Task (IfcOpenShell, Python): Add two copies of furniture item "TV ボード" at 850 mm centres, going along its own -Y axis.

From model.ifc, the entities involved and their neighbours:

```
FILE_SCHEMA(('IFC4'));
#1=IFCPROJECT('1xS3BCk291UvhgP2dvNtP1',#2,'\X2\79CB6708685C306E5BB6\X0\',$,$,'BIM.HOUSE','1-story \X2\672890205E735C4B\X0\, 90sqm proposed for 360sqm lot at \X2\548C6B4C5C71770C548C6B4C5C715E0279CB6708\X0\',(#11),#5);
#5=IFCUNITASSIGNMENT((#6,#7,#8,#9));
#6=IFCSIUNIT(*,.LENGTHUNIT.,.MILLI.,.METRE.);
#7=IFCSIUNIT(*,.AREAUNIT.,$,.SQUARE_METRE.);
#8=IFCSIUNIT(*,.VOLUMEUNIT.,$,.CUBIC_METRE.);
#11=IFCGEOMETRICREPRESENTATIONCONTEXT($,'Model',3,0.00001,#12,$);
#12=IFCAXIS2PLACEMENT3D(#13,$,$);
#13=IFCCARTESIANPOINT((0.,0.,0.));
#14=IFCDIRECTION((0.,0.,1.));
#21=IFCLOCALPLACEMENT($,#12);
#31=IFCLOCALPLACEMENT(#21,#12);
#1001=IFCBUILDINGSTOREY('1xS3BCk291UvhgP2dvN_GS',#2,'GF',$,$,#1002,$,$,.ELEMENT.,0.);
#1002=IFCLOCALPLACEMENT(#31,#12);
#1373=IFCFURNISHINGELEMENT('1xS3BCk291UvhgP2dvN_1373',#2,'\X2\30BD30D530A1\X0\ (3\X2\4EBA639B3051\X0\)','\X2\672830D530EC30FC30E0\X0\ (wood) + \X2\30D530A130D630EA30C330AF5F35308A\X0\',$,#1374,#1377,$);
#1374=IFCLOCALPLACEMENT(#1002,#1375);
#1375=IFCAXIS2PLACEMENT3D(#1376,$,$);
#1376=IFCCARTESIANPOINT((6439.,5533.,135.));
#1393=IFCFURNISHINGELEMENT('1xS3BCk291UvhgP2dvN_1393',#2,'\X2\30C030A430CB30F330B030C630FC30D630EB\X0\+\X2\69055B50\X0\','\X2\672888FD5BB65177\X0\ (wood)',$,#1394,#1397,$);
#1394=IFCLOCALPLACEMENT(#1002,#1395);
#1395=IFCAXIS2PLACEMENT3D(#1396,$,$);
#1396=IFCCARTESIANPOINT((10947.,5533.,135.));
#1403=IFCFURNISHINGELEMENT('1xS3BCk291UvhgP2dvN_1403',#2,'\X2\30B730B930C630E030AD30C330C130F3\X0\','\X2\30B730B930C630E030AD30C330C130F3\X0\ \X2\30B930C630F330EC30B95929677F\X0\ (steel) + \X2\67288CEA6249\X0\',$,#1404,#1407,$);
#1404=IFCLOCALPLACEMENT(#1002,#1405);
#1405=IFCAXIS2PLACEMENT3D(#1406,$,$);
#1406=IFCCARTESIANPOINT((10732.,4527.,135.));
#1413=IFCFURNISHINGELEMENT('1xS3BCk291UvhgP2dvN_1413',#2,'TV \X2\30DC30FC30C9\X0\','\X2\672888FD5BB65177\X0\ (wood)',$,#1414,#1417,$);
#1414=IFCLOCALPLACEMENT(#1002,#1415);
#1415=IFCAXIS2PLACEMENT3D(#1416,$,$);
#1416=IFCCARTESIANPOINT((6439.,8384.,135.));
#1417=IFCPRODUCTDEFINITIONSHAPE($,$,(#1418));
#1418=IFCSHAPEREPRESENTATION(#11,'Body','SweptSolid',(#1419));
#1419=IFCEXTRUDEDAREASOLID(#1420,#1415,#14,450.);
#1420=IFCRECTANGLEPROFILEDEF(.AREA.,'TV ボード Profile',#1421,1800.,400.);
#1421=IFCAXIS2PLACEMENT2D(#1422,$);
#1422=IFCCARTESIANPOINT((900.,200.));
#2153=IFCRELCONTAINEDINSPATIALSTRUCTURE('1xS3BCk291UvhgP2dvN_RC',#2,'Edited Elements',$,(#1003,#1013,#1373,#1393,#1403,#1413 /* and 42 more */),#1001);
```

```python
import ifcopenshell
import ifcopenshell.api.geometry
import ifcopenshell.api.root
import ifcopenshell.util.element
import ifcopenshell.util.placement

model = ifcopenshell.open("model.ifc")


def reuse_history(source, copy):
    """copy_class also copies each property set's owner history, people and application; keep the originals."""
    for rel in copy.IsDefinedBy:
        if rel.is_a("IfcRelDefinesByProperties") and (history := rel.RelatingPropertyDefinition.OwnerHistory):
            rel.RelatingPropertyDefinition.OwnerHistory = source.OwnerHistory
            ifcopenshell.util.element.remove_deep2(model, history)


source = model.by_id(1413)
base = ifcopenshell.util.placement.get_local_placement(source.ObjectPlacement)
step = -base[:3, 1] * 850.0

for i in range(1, 3):
    copy = ifcopenshell.api.root.copy_class(model, product=source)
    copy.Representation = ifcopenshell.util.element.copy_deep(
        model, source.Representation, exclude=["IfcGeometricRepresentationContext", "IfcRepresentationMap"]
    )
    reuse_history(source, copy)
    matrix = base.copy()
    matrix[:3, 3] += i * step
    print("added at", matrix[:3, 3].round(3) + 0.0)
    ifcopenshell.api.geometry.edit_object_placement(model, product=copy, matrix=matrix, is_si=False)

model.write("model_rev.ifc")
```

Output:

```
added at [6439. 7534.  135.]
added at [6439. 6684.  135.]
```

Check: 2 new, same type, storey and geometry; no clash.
